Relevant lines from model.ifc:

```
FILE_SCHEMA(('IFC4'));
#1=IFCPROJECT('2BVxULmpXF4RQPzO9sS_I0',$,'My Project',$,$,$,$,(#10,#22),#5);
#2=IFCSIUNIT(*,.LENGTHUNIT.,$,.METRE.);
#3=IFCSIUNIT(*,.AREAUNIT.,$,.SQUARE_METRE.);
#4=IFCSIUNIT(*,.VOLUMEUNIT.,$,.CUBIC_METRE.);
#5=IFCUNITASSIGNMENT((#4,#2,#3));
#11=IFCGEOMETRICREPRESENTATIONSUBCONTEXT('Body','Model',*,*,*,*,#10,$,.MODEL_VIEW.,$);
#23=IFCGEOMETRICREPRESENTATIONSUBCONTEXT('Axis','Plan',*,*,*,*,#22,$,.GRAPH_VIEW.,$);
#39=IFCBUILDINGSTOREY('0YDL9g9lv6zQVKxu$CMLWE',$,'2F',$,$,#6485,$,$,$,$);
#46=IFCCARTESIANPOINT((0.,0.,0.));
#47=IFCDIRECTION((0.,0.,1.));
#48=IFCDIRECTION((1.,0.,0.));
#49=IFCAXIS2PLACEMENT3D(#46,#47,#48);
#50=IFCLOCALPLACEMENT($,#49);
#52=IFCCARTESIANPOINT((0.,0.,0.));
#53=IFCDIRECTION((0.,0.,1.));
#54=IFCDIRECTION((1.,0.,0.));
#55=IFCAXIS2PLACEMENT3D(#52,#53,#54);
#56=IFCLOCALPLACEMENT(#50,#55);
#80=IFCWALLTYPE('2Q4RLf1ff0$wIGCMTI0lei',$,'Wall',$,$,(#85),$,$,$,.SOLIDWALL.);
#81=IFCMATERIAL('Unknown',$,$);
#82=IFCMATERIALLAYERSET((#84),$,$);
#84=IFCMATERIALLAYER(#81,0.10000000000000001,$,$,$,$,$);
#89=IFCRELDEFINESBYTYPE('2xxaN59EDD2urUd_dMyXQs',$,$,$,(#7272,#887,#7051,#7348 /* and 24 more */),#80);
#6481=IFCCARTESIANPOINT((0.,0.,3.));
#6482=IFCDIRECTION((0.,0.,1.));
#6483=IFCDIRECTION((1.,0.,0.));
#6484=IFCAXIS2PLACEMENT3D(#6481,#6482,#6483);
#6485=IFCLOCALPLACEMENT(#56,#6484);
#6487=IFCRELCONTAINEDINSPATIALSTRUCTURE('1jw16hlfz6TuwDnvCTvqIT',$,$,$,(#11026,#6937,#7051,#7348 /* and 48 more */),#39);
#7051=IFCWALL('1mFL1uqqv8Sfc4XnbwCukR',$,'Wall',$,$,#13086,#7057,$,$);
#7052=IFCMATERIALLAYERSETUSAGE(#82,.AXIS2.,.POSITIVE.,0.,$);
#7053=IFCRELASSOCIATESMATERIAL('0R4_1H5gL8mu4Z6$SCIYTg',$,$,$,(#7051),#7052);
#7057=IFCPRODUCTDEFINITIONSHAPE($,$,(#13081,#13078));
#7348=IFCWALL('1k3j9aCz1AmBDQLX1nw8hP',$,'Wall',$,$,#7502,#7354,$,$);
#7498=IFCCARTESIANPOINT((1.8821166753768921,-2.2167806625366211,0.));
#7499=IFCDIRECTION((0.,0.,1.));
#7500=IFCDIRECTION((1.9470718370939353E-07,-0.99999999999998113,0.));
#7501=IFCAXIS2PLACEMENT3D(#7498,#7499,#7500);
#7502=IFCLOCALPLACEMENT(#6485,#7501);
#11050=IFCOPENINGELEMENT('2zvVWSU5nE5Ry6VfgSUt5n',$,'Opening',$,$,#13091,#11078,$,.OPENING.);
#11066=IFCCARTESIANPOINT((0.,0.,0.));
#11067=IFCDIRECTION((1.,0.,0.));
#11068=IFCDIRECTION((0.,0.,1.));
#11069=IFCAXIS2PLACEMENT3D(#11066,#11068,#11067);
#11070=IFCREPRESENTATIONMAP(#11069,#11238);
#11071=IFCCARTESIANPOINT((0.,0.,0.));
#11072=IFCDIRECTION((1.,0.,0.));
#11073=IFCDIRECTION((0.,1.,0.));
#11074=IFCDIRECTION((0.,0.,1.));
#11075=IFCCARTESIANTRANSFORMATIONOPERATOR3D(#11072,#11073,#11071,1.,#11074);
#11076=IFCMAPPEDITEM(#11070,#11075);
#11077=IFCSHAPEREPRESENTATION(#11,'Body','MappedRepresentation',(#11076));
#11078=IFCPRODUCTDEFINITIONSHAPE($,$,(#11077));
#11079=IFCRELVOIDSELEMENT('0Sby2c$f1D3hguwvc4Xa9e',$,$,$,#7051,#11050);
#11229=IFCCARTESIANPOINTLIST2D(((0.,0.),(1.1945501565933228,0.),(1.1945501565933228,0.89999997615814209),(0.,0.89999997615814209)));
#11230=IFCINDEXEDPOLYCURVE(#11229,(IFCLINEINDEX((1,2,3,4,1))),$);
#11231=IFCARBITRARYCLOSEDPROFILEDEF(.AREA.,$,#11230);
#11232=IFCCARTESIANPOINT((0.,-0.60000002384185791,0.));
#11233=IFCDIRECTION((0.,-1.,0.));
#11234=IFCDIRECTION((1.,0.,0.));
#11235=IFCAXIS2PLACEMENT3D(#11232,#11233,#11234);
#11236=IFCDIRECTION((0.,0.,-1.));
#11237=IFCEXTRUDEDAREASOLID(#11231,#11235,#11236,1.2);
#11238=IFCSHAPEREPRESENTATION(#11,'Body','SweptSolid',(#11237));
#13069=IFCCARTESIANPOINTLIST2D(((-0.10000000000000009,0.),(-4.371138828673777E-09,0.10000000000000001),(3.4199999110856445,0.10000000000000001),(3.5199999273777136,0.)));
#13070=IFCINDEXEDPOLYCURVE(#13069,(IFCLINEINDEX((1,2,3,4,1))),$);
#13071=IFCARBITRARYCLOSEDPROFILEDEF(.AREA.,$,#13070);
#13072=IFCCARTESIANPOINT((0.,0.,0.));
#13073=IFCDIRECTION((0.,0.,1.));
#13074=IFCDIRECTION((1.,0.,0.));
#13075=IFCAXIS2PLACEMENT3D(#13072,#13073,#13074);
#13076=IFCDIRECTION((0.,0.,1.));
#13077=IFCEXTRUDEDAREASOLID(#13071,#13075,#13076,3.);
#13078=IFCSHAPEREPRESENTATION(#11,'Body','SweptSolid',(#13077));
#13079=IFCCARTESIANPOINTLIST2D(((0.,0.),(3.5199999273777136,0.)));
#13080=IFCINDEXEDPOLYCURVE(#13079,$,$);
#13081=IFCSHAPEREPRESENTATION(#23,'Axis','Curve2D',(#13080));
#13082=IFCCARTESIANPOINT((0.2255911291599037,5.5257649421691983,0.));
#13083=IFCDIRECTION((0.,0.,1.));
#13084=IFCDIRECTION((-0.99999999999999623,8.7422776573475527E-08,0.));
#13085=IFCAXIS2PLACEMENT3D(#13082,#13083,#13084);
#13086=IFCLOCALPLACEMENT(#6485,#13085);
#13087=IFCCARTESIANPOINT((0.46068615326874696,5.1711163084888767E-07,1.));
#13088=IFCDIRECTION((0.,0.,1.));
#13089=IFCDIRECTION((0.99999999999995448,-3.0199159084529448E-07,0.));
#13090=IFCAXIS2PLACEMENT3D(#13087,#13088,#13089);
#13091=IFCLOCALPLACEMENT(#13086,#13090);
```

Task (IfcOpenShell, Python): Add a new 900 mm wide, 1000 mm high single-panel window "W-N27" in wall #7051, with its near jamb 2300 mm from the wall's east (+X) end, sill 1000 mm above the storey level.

```python
import numpy as np
import ifcopenshell
import ifcopenshell.api.feature
import ifcopenshell.api.geometry
import ifcopenshell.api.root
import ifcopenshell.api.spatial
import ifcopenshell.geom
import ifcopenshell.util.element
import ifcopenshell.util.placement
import ifcopenshell.util.representation
import ifcopenshell.util.shape
import ifcopenshell.util.unit

model = ifcopenshell.open("model.ifc")
unit_scale = ifcopenshell.util.unit.calculate_unit_scale(model)
settings = ifcopenshell.geom.settings()


def volume(element):
    """Net volume in cubic metres, openings subtracted."""
    shape = ifcopenshell.geom.create_shape(settings, element)
    return ifcopenshell.util.shape.get_volume(shape.geometry)


wall = model.by_guid("1mFL1uqqv8Sfc4XnbwCukR")
storey = ifcopenshell.util.element.get_container(wall, ifc_class="IfcBuildingStorey")
context = ifcopenshell.util.representation.get_context(model, "Model", "Body", "MODEL_VIEW")
before = volume(wall)

width, height, from_end, sill = 0.9, 1, 2.3, 1  # metres

# The wall runs along its own X axis, and the end named is its -X end.
wall_shape = ifcopenshell.geom.create_shape(settings, wall)
x, y, z = ifcopenshell.util.shape.get_vertices(wall_shape.geometry).T
start = x.min() + from_end
face, thickness = float(y.min()), float(y.max() - y.min())
wall_matrix = ifcopenshell.util.placement.get_local_placement(wall.ObjectPlacement)
level = ifcopenshell.util.placement.get_local_placement(storey.ObjectPlacement)[2, 3]


def in_wall(x, y):
    """Placement at x, y metres in the wall's axes, at sill height."""
    matrix = wall_matrix.copy()
    matrix[:, 3] = wall_matrix @ np.array([x / unit_scale, y / unit_scale, 0.0, 1.0])
    matrix[2, 3] = level + sill / unit_scale
    return matrix


# Opening: a box that overshoots both wall faces by 50 mm.
opening = ifcopenshell.api.root.create_entity(model, ifc_class="IfcOpeningElement", predefined_type="OPENING")
box = ifcopenshell.api.geometry.add_wall_representation(
    model, context=context, length=width, height=height, thickness=thickness + 0.1
)
ifcopenshell.api.geometry.assign_representation(model, product=opening, representation=box)
ifcopenshell.api.geometry.edit_object_placement(model, product=opening, matrix=in_wall(start, face - 0.05), is_si=False)
ifcopenshell.api.feature.add_feature(model, feature=opening, element=wall)

window = ifcopenshell.api.root.create_entity(model, ifc_class="IfcWindow", name="W-N27", predefined_type="WINDOW")
window.OverallWidth, window.OverallHeight = width / unit_scale, height / unit_scale
window.PartitioningType = "SINGLE_PANEL"
body = ifcopenshell.api.geometry.add_window_representation(
    model,
    context=context,
    overall_width=window.OverallWidth,
    overall_height=window.OverallHeight,
    partition_type="SINGLE_PANEL",
)
ifcopenshell.api.geometry.assign_representation(model, product=window, representation=body)
ifcopenshell.api.spatial.assign_container(model, products=[window], relating_structure=storey)
ifcopenshell.api.feature.add_filling(model, opening=opening, element=window)

# Centre the window in the wall's thickness.
ifcopenshell.api.geometry.edit_object_placement(model, product=window, matrix=in_wall(start, face), is_si=False)
window_shape = ifcopenshell.geom.create_shape(settings, window)
depth = ifcopenshell.util.shape.get_vertices(window_shape.geometry)[:, 1]
offset = face + thickness / 2 - (depth.min() + depth.max()) / 2
ifcopenshell.api.geometry.edit_object_placement(model, product=window, matrix=in_wall(start, offset), is_si=False)

after = volume(wall)

print(f"wall volume {before:.3f} -> {after:.3f} m3")

model.write("model-out.ifc")
```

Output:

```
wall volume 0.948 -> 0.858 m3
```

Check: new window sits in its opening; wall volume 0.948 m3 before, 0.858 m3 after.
